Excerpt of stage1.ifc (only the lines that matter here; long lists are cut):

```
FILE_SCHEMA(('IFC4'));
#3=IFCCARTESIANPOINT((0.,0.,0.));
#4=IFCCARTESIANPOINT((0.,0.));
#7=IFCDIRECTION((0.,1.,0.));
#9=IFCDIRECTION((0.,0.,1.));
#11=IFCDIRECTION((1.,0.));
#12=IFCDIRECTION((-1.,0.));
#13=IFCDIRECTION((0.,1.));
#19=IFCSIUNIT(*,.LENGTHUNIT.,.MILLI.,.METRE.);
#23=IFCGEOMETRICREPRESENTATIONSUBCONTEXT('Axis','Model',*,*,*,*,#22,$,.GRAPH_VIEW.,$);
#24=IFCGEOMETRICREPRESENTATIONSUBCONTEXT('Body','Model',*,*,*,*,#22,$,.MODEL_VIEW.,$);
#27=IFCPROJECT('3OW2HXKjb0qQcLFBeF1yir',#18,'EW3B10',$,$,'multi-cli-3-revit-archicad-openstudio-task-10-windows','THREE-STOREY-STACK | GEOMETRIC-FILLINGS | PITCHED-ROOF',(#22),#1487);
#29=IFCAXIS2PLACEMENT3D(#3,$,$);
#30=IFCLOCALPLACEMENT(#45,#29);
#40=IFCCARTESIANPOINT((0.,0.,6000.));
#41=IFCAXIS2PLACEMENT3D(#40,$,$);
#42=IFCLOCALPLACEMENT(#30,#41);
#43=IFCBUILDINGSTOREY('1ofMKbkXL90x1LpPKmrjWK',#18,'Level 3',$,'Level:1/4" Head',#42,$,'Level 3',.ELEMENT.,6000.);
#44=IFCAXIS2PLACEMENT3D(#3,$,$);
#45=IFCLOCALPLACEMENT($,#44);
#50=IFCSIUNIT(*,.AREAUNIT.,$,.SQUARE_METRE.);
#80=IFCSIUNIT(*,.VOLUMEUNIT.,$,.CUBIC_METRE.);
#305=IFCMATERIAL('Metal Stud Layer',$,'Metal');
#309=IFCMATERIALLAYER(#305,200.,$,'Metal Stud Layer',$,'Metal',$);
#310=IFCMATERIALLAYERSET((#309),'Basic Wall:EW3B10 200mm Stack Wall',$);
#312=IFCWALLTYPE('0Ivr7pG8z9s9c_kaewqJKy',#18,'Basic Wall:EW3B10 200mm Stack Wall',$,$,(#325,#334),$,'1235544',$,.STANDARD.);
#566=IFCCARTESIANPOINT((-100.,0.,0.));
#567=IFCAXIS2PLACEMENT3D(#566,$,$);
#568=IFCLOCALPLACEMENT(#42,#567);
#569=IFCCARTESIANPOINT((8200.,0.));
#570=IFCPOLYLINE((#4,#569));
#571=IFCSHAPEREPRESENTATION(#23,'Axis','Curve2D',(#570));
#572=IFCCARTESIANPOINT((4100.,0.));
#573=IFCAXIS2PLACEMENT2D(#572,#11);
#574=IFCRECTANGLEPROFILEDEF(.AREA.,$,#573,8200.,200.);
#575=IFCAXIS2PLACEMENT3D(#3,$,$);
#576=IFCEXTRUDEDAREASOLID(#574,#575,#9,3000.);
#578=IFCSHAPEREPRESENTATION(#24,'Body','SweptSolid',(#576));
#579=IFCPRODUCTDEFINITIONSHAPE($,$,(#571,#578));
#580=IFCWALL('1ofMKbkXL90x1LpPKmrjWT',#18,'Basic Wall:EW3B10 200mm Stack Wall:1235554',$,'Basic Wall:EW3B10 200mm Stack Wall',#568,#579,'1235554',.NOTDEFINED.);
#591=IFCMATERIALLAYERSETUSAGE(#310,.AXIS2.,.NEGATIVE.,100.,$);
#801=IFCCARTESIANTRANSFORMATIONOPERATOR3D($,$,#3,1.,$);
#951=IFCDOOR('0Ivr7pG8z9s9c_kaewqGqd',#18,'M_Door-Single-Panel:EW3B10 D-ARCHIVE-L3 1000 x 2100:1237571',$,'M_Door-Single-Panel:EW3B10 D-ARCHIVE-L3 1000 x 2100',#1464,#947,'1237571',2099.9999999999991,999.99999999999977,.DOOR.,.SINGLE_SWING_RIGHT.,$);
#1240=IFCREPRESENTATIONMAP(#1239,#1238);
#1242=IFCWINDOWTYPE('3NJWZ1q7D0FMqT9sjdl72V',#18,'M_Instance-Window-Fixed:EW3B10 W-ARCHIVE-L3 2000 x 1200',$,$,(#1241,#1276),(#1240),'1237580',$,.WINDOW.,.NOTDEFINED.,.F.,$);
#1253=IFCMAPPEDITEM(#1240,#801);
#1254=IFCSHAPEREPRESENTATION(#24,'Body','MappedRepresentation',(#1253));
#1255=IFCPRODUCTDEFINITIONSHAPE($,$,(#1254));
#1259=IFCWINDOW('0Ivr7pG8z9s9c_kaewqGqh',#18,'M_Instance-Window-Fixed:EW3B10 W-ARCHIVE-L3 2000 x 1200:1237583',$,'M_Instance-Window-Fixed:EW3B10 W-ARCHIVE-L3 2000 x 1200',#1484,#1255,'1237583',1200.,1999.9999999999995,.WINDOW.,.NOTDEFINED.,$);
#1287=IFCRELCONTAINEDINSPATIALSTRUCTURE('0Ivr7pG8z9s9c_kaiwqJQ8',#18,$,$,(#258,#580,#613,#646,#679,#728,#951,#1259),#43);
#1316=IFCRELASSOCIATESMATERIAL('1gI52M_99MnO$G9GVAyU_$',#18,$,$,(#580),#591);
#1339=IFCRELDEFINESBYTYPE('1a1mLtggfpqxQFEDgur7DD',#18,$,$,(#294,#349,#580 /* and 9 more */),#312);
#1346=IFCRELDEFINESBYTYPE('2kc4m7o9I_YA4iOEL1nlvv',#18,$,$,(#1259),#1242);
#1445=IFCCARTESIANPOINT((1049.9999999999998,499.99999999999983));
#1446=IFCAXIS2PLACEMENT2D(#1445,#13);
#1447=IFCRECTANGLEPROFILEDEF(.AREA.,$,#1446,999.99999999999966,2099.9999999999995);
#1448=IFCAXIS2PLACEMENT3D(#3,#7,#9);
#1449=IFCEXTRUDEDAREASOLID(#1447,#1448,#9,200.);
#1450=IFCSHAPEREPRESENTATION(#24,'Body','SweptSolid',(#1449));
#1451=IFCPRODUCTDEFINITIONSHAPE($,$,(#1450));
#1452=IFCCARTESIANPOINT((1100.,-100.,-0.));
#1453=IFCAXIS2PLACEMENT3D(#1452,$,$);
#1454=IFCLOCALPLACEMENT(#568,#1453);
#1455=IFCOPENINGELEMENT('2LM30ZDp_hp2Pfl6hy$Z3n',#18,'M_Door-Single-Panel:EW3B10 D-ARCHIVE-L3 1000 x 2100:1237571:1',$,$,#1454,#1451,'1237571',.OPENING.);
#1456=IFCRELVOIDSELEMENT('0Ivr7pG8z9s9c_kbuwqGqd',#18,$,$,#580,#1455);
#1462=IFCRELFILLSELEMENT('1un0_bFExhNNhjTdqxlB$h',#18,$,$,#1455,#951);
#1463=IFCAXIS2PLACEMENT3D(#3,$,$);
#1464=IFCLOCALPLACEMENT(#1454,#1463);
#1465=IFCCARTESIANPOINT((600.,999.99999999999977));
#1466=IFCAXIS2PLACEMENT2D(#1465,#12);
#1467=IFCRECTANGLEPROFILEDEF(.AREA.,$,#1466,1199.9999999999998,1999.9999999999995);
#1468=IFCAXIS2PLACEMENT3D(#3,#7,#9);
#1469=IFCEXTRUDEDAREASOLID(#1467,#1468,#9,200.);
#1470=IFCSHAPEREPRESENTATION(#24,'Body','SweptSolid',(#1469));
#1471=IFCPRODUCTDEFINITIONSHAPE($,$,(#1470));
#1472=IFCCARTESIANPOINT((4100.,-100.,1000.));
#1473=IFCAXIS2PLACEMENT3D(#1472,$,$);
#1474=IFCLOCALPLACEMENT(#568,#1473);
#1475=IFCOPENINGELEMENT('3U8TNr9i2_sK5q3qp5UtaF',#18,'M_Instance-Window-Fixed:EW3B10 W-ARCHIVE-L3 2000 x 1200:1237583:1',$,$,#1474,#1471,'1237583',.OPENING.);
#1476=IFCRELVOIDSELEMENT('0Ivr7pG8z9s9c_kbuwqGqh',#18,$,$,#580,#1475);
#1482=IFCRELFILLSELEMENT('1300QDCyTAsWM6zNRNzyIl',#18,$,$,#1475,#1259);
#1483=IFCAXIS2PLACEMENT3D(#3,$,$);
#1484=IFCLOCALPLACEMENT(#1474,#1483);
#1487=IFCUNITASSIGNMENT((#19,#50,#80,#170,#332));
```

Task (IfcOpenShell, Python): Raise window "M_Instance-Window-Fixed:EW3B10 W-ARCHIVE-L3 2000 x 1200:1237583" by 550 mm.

```python
import numpy as np
import ifcopenshell
import ifcopenshell.api.geometry
import ifcopenshell.util.placement
import ifcopenshell.util.unit

model = ifcopenshell.open("stage1.ifc")
unit_scale = ifcopenshell.util.unit.calculate_unit_scale(model)

window = model.by_id(1259)
opening = window.FillsVoids[0].RelatingOpeningElement
dz = 550.0

shift = np.array([0.0, 0.0, dz])
# The window is placed relative to its opening, so it follows when the opening moves.
matrix = ifcopenshell.util.placement.get_local_placement(opening.ObjectPlacement)
matrix[:3, 3] += shift
ifcopenshell.api.geometry.edit_object_placement(
    model, product=opening, matrix=matrix, is_si=False, should_transform_children=True
)

print(f"moved by {dz * unit_scale:+.3f} m")

model.write("stage1_edited.ifc")
```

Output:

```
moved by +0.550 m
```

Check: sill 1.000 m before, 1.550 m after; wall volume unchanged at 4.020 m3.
